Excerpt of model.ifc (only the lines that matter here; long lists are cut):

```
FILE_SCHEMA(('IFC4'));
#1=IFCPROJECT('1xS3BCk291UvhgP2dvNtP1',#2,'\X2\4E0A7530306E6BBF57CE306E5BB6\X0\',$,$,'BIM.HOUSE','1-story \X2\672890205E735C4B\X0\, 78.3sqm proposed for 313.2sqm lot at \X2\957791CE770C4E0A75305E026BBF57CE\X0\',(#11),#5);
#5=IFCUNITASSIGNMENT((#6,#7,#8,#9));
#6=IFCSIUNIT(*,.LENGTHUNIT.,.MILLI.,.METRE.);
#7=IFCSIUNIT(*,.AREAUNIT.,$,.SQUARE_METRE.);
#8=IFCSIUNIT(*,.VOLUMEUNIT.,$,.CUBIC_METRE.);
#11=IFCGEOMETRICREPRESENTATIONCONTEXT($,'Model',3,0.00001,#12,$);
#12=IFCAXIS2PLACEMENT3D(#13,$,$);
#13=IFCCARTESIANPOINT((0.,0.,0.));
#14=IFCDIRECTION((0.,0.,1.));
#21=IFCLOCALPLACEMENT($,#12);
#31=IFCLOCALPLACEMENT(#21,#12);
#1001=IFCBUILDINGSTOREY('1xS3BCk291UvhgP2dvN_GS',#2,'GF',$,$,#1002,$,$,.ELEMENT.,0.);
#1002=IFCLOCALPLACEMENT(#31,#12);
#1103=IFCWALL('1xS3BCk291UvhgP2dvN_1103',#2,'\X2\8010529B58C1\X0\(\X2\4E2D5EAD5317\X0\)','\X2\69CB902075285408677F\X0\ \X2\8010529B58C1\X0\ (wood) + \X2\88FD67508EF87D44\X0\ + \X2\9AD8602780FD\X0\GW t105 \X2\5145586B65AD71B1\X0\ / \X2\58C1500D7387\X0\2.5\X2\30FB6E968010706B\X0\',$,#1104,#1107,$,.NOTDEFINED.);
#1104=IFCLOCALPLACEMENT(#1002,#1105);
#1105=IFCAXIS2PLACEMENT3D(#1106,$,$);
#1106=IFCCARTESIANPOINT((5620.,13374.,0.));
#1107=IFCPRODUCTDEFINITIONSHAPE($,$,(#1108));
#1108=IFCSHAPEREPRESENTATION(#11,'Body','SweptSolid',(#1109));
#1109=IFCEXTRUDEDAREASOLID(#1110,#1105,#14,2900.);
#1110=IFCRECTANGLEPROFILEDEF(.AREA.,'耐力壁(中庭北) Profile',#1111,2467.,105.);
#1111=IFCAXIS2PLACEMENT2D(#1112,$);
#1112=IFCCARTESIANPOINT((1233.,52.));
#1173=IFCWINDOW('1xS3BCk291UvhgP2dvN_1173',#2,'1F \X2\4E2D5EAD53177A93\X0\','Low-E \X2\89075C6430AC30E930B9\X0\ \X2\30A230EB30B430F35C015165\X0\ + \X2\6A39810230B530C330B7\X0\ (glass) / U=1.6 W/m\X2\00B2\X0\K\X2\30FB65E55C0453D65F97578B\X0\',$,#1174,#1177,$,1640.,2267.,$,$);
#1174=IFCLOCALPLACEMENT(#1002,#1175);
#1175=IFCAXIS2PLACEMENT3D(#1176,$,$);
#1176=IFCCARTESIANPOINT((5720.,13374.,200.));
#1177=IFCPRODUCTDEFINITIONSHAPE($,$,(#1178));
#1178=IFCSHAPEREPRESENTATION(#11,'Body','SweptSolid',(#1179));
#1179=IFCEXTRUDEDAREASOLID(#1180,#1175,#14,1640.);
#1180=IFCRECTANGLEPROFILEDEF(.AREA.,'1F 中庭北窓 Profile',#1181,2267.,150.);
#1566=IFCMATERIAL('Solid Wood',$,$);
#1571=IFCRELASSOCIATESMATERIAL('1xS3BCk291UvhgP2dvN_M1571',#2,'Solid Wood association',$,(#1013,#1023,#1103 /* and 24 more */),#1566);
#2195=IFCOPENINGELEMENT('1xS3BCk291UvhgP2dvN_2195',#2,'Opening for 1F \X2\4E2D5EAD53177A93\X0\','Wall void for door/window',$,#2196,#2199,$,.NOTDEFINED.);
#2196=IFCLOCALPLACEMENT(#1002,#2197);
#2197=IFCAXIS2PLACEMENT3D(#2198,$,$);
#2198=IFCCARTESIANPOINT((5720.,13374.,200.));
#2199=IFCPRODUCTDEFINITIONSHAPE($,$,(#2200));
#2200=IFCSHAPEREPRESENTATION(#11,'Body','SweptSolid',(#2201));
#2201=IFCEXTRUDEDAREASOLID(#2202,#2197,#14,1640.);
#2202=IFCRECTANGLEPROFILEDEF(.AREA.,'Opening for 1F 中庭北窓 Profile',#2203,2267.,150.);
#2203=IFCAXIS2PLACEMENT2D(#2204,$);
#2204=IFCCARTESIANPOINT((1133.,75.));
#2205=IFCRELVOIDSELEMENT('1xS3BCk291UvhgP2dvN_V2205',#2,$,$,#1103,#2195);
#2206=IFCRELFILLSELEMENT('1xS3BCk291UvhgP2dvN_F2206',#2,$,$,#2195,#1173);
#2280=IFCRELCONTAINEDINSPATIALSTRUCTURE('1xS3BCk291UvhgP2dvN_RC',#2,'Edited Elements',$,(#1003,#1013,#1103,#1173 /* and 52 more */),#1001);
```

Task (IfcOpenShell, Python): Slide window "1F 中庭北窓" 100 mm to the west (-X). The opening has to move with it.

```python
import ifcopenshell
import ifcopenshell.api.geometry
import ifcopenshell.util.placement
import ifcopenshell.util.unit

model = ifcopenshell.open("model.ifc")
unit_scale = ifcopenshell.util.unit.calculate_unit_scale(model)

window = model.by_guid("1xS3BCk291UvhgP2dvN_1173")
opening = window.FillsVoids[0].RelatingOpeningElement
wall = opening.VoidsElements[0].RelatingBuildingElement

wall_matrix = ifcopenshell.util.placement.get_local_placement(wall.ObjectPlacement)
shift = wall_matrix[:3, 0] * -0.1 / unit_scale
before = ifcopenshell.util.placement.get_local_placement(window.ObjectPlacement)[:3, 3].copy()

# The window is not placed relative to its opening, so move both.
for product in (opening, window):
    matrix = ifcopenshell.util.placement.get_local_placement(product.ObjectPlacement)
    matrix[:3, 3] += shift
    ifcopenshell.api.geometry.edit_object_placement(model, product=product, matrix=matrix, is_si=False)

after = ifcopenshell.util.placement.get_local_placement(window.ObjectPlacement)[:3, 3]
print("window moved by", (after - before).round(3) + 0.0)

model.write("model_edited.ifc")
```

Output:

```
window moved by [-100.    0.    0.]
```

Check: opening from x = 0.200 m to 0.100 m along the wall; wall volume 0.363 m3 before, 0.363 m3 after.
